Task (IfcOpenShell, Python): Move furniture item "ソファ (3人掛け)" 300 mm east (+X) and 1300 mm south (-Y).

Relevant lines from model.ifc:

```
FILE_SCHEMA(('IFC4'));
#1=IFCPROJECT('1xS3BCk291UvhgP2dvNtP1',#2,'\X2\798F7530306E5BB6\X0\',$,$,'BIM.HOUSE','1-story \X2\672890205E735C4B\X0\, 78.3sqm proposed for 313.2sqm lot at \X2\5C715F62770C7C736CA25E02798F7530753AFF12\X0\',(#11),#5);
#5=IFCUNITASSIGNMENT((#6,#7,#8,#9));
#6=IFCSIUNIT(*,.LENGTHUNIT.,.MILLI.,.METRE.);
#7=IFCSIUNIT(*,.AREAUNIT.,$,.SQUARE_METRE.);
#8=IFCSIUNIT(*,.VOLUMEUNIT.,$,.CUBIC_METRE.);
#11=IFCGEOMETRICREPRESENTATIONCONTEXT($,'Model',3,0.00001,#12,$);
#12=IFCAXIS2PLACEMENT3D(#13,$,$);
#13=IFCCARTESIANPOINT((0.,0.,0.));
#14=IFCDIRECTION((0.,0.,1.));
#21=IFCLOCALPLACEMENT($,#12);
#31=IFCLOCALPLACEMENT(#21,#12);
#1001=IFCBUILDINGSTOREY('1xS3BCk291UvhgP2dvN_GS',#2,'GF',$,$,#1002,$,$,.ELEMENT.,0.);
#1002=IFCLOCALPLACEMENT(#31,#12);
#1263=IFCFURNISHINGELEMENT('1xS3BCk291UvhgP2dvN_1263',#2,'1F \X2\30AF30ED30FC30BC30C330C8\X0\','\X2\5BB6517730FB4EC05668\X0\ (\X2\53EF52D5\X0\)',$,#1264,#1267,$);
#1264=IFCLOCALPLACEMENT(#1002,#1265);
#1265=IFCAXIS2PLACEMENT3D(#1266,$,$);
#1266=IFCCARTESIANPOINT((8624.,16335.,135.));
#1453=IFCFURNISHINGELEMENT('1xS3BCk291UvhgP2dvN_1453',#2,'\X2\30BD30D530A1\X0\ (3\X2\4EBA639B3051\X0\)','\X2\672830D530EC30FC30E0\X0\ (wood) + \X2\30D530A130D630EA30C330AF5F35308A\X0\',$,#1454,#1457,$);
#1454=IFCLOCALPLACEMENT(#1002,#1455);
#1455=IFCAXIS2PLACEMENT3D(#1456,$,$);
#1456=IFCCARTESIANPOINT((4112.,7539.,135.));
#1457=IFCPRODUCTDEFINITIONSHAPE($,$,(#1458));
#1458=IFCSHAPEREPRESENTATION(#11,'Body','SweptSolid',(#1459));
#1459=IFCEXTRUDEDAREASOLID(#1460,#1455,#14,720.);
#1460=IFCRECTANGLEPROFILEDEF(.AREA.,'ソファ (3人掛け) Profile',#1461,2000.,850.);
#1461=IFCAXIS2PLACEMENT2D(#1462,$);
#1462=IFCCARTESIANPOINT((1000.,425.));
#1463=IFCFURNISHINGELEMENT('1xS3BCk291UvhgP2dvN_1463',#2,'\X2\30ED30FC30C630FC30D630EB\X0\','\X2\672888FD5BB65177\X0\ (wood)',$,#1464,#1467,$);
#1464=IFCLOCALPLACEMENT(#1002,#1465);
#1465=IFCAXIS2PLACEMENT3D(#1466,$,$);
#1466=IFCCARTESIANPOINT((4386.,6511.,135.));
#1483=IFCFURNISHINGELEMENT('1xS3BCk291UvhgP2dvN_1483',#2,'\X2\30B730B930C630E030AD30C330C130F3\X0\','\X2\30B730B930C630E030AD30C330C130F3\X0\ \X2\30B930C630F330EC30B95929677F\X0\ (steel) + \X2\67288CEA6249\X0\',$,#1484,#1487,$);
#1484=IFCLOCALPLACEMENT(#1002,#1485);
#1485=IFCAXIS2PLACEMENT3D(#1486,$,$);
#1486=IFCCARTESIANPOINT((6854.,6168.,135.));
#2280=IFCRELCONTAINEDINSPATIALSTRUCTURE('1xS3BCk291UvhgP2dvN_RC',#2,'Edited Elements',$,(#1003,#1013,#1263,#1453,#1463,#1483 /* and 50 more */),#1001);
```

```python
import ifcopenshell
import ifcopenshell.api.geometry
import ifcopenshell.util.placement
import ifcopenshell.util.unit

model = ifcopenshell.open("model.ifc")
unit_scale = ifcopenshell.util.unit.calculate_unit_scale(model)

item = model.by_guid("1xS3BCk291UvhgP2dvN_1453")
matrix = ifcopenshell.util.placement.get_local_placement(item.ObjectPlacement)
matrix[0, 3] += 0.3 / unit_scale
matrix[1, 3] -= 1.3 / unit_scale
ifcopenshell.api.geometry.edit_object_placement(model, product=item, matrix=matrix, is_si=False)

print(ifcopenshell.util.placement.get_local_placement(item.ObjectPlacement).round(3) + 0.0)

model.write("model-out.ifc")
```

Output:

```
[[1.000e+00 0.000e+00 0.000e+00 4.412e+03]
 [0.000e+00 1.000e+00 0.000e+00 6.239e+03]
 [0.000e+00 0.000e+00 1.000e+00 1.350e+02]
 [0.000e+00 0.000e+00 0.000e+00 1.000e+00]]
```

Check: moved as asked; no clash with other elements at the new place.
